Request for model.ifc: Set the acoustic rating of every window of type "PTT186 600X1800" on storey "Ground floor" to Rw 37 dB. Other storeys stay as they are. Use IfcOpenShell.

First a look at what the model holds.

```python
import ifcopenshell
import ifcopenshell.util.element

model = ifcopenshell.open("model.ifc")
print(model.schema)
storey = next(s for s in model.by_type("IfcBuildingStorey") if s.Name == "Ground floor")
windows = [e for e in ifcopenshell.util.element.get_decomposition(storey) if e.is_a("IfcWindow")]
seen = {}
for e in windows:
    element_type = ifcopenshell.util.element.get_type(e)
    key = (element_type.Name if element_type != e and element_type else None, ifcopenshell.util.element.get_pset(e, "Pset_WindowCommon", "AcousticRating"))
    seen[key] = seen.get(key, 0) + 1
for (name, value), count in sorted(seen.items(), key=str):
    print(count, "x", name, "|", value)
```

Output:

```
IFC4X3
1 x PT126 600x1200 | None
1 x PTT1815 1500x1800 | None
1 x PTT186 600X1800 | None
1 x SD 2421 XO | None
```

```python
import ifcopenshell
import ifcopenshell.api.pset
import ifcopenshell.util.element

model = ifcopenshell.open("model.ifc")

storey = next(s for s in model.by_type("IfcBuildingStorey") if s.Name == "Ground floor")
windows = [e for e in ifcopenshell.util.element.get_decomposition(storey) if e.is_a("IfcWindow")]

count = 0
for e in windows:
    element_type = ifcopenshell.util.element.get_type(e)
    if element_type in (None, e) or element_type.Name != "PTT186 600X1800":
        continue
    # add_pset returns the element's existing set when there is one.
    pset = ifcopenshell.api.pset.add_pset(model, product=e, name="Pset_WindowCommon")
    ifcopenshell.api.pset.edit_pset(model, pset=pset, properties={"AcousticRating": "Rw 37 dB"})
    count += 1

print(count, "windows updated")

model.write("model-out.ifc")
```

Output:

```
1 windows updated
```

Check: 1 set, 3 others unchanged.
